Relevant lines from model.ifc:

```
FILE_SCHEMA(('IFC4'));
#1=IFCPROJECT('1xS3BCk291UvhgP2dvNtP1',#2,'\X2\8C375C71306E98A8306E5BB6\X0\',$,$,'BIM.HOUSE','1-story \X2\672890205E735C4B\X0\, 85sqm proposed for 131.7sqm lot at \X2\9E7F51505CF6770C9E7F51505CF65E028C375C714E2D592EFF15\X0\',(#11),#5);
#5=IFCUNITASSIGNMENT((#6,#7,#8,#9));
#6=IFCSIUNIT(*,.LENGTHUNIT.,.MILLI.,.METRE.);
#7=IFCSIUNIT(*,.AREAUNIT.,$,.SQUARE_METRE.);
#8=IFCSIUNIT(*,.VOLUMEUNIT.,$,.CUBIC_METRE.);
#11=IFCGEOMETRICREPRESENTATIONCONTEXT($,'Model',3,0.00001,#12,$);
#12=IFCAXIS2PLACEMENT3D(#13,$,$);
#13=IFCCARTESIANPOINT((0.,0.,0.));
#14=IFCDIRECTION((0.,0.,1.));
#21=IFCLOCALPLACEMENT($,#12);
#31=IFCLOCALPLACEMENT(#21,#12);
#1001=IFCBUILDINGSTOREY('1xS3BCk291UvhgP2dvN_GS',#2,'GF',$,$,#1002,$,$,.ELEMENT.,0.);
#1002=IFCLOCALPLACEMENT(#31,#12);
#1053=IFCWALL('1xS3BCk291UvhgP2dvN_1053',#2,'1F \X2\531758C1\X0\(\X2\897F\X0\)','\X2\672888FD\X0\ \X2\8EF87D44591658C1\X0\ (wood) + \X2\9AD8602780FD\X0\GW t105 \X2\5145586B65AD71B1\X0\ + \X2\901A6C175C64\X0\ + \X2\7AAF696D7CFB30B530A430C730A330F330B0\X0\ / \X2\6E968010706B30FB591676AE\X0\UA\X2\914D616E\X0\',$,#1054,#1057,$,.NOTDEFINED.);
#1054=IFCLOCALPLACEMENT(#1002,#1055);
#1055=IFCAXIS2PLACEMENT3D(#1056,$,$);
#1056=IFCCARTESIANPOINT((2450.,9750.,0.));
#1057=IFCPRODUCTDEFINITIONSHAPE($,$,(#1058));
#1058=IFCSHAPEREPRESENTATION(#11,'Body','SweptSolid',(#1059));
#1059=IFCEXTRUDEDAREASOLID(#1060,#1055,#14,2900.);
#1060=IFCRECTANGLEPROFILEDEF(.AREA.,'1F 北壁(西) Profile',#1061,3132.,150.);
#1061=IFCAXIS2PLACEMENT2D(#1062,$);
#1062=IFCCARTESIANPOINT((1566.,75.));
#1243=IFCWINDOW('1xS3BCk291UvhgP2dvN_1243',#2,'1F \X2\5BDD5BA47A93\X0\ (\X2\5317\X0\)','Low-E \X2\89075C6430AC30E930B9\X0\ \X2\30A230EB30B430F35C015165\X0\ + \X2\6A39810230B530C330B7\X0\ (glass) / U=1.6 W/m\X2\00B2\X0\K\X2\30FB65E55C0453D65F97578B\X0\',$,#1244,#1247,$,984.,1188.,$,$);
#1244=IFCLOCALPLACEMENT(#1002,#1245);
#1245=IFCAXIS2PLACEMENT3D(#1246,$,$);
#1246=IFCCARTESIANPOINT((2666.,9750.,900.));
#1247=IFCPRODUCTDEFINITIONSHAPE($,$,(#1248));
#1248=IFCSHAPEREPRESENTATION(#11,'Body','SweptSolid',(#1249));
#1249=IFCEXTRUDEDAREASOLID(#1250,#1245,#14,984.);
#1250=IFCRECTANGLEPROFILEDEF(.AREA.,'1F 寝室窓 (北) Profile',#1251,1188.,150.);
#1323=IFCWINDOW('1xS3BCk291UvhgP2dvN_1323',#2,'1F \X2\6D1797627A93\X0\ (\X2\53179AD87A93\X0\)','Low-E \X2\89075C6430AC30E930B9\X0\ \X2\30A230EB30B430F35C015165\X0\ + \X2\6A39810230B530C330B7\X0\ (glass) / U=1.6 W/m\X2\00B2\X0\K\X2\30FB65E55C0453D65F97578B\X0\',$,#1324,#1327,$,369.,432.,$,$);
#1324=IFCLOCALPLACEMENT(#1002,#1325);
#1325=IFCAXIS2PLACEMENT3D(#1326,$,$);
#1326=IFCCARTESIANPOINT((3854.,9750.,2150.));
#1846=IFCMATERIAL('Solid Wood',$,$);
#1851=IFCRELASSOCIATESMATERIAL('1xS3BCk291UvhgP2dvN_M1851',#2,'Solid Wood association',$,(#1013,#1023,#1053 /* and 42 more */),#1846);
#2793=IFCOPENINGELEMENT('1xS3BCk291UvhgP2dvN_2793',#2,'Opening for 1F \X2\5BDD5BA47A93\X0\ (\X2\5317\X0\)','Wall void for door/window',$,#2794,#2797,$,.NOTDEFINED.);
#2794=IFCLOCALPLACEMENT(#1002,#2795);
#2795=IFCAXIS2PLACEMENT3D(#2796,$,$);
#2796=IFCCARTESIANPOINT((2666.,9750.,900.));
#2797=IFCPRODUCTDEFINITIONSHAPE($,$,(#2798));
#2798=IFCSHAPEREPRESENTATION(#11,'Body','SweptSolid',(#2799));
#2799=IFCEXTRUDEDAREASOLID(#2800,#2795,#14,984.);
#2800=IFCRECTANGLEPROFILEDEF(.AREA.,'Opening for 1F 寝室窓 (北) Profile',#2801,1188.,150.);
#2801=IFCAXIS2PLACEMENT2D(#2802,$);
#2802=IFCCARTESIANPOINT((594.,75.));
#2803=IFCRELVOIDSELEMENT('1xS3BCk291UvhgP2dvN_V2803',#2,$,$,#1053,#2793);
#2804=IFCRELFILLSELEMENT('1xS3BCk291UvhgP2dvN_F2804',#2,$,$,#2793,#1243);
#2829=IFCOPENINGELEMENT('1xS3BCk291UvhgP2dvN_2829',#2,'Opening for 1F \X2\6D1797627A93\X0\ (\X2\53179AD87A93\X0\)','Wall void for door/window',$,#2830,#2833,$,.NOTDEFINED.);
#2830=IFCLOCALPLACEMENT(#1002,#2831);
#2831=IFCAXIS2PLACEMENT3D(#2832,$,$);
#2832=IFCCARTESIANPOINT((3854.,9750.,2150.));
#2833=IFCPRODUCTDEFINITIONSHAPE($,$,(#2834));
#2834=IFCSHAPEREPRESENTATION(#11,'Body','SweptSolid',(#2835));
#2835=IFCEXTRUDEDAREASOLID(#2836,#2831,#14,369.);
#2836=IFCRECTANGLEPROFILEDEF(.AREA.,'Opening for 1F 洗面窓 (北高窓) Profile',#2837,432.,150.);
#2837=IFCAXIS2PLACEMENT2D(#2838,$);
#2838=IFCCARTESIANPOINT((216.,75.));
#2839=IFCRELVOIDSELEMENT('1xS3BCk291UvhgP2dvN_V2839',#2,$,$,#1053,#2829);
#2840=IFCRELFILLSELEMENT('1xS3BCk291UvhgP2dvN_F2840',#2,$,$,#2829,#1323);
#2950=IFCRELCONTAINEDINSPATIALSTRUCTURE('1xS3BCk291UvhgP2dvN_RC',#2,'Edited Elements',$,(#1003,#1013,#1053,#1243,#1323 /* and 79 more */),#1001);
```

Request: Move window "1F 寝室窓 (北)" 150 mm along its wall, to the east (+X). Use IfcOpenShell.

```python
import ifcopenshell
import ifcopenshell.api.geometry
import ifcopenshell.util.placement
import ifcopenshell.util.unit

model = ifcopenshell.open("model.ifc")
unit_scale = ifcopenshell.util.unit.calculate_unit_scale(model)

window = model.by_guid("1xS3BCk291UvhgP2dvN_1243")
opening = window.FillsVoids[0].RelatingOpeningElement
wall = opening.VoidsElements[0].RelatingBuildingElement

wall_matrix = ifcopenshell.util.placement.get_local_placement(wall.ObjectPlacement)
shift = wall_matrix[:3, 0] * 0.15 / unit_scale
before = ifcopenshell.util.placement.get_local_placement(window.ObjectPlacement)[:3, 3].copy()

# The window is not placed relative to its opening, so move both.
for product in (opening, window):
    matrix = ifcopenshell.util.placement.get_local_placement(product.ObjectPlacement)
    matrix[:3, 3] += shift
    ifcopenshell.api.geometry.edit_object_placement(model, product=product, matrix=matrix, is_si=False)

after = ifcopenshell.util.placement.get_local_placement(window.ObjectPlacement)[:3, 3]
print("window moved by", (after - before).round(3) + 0.0)

model.write("model_v2.ifc")
```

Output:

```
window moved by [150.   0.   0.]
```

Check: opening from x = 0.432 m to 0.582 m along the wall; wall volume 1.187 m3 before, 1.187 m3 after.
